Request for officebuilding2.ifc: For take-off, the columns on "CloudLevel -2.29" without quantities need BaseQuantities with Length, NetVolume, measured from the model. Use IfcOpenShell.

First a look at what the model holds.

```python
import ifcopenshell
import ifcopenshell.util.element
import ifcopenshell.util.unit

model = ifcopenshell.open("officebuilding2.ifc")
print(model.schema)
for unit_type in ("LENGTHUNIT", "AREAUNIT", "VOLUMEUNIT"):
    print(unit_type, ifcopenshell.util.unit.calculate_unit_scale(model, unit_type))
storey = next(s for s in model.by_type("IfcBuildingStorey") if s.Name == "CloudLevel -2.29")
columns = [e for e in ifcopenshell.util.element.get_decomposition(storey) if e.is_a("IfcColumn")]
for e in sorted(columns, key=lambda e: e.id()):
    print(e.id(), e.is_a(), e.Name, list(ifcopenshell.util.element.get_psets(e, qtos_only=True)), sep=" | ")
```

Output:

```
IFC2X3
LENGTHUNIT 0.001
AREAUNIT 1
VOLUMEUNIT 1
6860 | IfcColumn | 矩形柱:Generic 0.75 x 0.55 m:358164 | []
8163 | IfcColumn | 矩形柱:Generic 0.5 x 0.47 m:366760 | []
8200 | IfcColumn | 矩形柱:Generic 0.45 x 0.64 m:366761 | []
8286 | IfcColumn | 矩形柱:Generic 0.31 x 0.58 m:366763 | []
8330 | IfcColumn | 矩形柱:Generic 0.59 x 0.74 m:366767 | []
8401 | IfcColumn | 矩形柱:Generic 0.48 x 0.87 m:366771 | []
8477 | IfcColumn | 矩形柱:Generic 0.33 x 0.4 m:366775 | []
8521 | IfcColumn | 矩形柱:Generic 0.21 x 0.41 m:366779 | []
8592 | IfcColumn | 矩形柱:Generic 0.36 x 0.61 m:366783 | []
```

```python
import ifcopenshell
import ifcopenshell.api.pset
import ifcopenshell.geom
import ifcopenshell.util.element
import ifcopenshell.util.shape
import ifcopenshell.util.unit

model = ifcopenshell.open("officebuilding2.ifc")
unit_scale = ifcopenshell.util.unit.calculate_unit_scale(model)
volume_scale = ifcopenshell.util.unit.calculate_unit_scale(model, "VOLUMEUNIT")
settings = ifcopenshell.geom.settings()

storey = next(s for s in model.by_type("IfcBuildingStorey") if s.Name == "CloudLevel -2.29")
columns = [e for e in ifcopenshell.util.element.get_decomposition(storey) if e.is_a("IfcColumn")]

for e in sorted(columns, key=lambda e: e.id()):
    if ifcopenshell.util.element.get_psets(e, qtos_only=True, should_inherit=False):
        continue
    # Geometry comes back in metres, in the element's own axes.
    shape = ifcopenshell.geom.create_shape(settings, e)
    values = {
        "Length": ifcopenshell.util.shape.get_z(shape.geometry) / unit_scale,
        "NetVolume": ifcopenshell.util.shape.get_volume(shape.geometry) / volume_scale,
    }
    qto = ifcopenshell.api.pset.add_qto(model, product=e, name="BaseQuantities")
    ifcopenshell.api.pset.edit_qto(model, qto=qto, properties=values)
    print(e.id(), {k: round(v, 3) for k, v in values.items()})

model.write("officebuilding2_v2.ifc")
```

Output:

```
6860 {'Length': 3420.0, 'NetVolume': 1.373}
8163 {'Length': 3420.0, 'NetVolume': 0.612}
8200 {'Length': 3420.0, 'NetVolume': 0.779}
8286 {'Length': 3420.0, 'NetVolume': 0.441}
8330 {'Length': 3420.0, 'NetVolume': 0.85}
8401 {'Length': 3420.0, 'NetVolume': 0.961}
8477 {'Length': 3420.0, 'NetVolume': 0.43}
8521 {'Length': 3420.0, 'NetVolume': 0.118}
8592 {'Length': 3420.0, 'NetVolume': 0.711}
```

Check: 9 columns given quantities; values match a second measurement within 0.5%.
